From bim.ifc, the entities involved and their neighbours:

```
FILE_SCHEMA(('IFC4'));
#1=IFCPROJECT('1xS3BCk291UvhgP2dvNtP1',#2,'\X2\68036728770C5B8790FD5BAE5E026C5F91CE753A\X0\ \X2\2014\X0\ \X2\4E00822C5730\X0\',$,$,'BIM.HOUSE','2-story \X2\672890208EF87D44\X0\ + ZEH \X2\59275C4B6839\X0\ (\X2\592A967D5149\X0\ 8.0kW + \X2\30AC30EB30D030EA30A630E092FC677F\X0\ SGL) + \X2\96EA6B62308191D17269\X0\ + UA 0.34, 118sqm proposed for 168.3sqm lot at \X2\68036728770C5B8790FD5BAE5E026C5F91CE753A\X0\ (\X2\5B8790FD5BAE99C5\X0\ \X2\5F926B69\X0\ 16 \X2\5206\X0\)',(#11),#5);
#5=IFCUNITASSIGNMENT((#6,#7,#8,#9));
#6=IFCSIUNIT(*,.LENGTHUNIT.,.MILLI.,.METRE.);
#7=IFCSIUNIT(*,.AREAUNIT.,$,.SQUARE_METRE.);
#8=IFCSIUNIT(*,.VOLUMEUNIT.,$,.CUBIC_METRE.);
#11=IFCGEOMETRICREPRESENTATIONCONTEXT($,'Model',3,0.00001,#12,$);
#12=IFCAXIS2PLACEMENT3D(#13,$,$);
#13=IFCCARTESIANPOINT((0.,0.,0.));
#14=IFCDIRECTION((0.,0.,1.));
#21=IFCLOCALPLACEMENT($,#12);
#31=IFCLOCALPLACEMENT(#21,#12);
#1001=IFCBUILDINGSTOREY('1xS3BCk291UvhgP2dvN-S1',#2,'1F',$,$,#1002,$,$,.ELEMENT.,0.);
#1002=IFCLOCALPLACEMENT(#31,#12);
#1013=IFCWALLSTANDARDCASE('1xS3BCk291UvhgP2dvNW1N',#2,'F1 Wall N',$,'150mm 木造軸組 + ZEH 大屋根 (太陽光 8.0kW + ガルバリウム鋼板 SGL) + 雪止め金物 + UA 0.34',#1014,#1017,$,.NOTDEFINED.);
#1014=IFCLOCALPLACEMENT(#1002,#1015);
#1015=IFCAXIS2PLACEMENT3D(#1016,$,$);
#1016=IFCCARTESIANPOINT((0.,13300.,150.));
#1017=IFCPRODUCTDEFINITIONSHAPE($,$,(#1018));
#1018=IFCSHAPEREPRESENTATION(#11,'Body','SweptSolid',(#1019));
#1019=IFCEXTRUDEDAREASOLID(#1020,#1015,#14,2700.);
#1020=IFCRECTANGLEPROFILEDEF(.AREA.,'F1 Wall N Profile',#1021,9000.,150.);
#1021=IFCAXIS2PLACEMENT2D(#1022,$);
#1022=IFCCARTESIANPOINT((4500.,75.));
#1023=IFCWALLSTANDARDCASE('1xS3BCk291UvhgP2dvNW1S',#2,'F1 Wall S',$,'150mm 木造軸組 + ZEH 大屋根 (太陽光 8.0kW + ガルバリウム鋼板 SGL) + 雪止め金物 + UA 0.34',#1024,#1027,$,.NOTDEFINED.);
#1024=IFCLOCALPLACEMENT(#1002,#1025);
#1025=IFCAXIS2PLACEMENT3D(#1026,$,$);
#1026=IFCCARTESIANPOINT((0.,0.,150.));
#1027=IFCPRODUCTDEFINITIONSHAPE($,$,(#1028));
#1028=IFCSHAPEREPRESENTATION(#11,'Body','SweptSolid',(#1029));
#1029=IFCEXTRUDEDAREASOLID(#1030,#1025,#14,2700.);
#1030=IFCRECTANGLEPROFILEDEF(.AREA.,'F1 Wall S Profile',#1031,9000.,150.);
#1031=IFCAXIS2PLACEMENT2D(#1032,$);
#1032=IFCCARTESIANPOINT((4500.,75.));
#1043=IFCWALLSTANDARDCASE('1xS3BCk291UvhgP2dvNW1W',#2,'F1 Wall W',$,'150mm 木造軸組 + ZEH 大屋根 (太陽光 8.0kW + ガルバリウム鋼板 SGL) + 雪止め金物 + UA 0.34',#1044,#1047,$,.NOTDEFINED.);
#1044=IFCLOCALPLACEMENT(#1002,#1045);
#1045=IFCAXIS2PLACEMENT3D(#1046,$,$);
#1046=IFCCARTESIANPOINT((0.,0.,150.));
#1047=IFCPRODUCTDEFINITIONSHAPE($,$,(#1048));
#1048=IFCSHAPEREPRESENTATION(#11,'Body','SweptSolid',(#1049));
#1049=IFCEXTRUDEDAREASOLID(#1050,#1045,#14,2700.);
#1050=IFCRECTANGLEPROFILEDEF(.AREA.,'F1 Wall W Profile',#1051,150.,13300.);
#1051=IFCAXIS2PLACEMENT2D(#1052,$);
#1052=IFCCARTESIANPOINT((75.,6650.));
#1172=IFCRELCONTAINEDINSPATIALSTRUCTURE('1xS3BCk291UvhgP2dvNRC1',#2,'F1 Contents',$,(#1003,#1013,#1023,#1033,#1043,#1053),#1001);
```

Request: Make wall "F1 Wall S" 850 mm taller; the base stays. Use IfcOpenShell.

```python
import ifcopenshell
import ifcopenshell.geom
import ifcopenshell.util.shape
import ifcopenshell.util.unit

model = ifcopenshell.open("bim.ifc")
unit_scale = ifcopenshell.util.unit.calculate_unit_scale(model)
settings = ifcopenshell.geom.settings()


def volume(element):
    """Net volume in cubic metres, openings subtracted."""
    shape = ifcopenshell.geom.create_shape(settings, element)
    return ifcopenshell.util.shape.get_volume(shape.geometry)


wall = model.by_guid("1xS3BCk291UvhgP2dvNW1S")
before = volume(wall)

body = next(r for r in wall.Representation.Representations if r.RepresentationIdentifier == "Body")
solid = body.Items[0]
old_height = solid.Depth
solid.Depth += 0.85 / unit_scale
after = volume(wall)

print(f"height {old_height:g} -> {solid.Depth:g}, volume {before:.3f} -> {after:.3f} m3")

model.write("bim_updated.ifc")
```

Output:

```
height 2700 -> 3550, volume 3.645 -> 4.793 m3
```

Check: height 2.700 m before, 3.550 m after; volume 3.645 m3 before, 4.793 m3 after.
